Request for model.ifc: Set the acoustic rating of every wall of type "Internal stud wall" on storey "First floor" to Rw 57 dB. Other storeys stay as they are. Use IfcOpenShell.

First a look at what the model holds.

```python
import ifcopenshell
import ifcopenshell.util.element

model = ifcopenshell.open("model.ifc")
print(model.schema)
storey = next(s for s in model.by_type("IfcBuildingStorey") if s.Name == "First floor")
walls = [e for e in ifcopenshell.util.element.get_decomposition(storey) if e.is_a("IfcWall")]
seen = {}
for e in walls:
    element_type = ifcopenshell.util.element.get_type(e)
    key = (element_type.Name if element_type != e and element_type else None, ifcopenshell.util.element.get_pset(e, "Pset_WallCommon", "AcousticRating"))
    seen[key] = seen.get(key, 0) + 1
for (name, value), count in sorted(seen.items(), key=str):
    print(count, "x", name, "|", value)
```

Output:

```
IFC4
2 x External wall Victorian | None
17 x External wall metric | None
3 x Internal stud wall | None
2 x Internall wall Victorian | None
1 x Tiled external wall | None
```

```python
import ifcopenshell
import ifcopenshell.api.pset
import ifcopenshell.util.element

model = ifcopenshell.open("model.ifc")

storey = next(s for s in model.by_type("IfcBuildingStorey") if s.Name == "First floor")
walls = [e for e in ifcopenshell.util.element.get_decomposition(storey) if e.is_a("IfcWall")]

count = 0
for e in walls:
    element_type = ifcopenshell.util.element.get_type(e)
    if element_type in (None, e) or element_type.Name != "Internal stud wall":
        continue
    # add_pset returns the element's existing set when there is one.
    pset = ifcopenshell.api.pset.add_pset(model, product=e, name="Pset_WallCommon")
    ifcopenshell.api.pset.edit_pset(model, pset=pset, properties={"AcousticRating": "Rw 57 dB"})
    count += 1

print(count, "walls updated")

model.write("model_v2.ifc")
```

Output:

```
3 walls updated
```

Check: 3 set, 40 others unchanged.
